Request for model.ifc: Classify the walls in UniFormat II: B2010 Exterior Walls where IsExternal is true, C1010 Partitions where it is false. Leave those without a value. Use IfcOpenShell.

First a look at what the model holds.

```python
import ifcopenshell
import ifcopenshell.util.element

model = ifcopenshell.open("model.ifc")
print(model.schema)
print("classifications:", [c.Name for c in model.by_type("IfcClassification")])
values = [ifcopenshell.util.element.get_pset(e, "Pset_WallCommon", "IsExternal") for e in model.by_type("IfcWall")]
for value in (True, False, None):
    print("IsExternal", value, values.count(value))
```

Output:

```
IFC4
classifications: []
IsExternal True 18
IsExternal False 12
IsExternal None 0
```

```python
import ifcopenshell
import ifcopenshell.api.classification
import ifcopenshell.util.element

model = ifcopenshell.open("model.ifc")

system = ifcopenshell.api.classification.add_classification(model, classification="UniFormat II")

walls = model.by_type("IfcWall")
external = {e: ifcopenshell.util.element.get_pset(e, "Pset_WallCommon", "IsExternal") for e in walls}
for flag, code, name in ((True, "B2010", "Exterior Walls"), (False, "C1010", "Partitions")):
    products = [e for e in walls if external[e] is flag]
    ifcopenshell.api.classification.add_reference(
        model, products=products, classification=system, identification=code, name=name
    )
    print(code, len(products))

model.write("model-out.ifc")
```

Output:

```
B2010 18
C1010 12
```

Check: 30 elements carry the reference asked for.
